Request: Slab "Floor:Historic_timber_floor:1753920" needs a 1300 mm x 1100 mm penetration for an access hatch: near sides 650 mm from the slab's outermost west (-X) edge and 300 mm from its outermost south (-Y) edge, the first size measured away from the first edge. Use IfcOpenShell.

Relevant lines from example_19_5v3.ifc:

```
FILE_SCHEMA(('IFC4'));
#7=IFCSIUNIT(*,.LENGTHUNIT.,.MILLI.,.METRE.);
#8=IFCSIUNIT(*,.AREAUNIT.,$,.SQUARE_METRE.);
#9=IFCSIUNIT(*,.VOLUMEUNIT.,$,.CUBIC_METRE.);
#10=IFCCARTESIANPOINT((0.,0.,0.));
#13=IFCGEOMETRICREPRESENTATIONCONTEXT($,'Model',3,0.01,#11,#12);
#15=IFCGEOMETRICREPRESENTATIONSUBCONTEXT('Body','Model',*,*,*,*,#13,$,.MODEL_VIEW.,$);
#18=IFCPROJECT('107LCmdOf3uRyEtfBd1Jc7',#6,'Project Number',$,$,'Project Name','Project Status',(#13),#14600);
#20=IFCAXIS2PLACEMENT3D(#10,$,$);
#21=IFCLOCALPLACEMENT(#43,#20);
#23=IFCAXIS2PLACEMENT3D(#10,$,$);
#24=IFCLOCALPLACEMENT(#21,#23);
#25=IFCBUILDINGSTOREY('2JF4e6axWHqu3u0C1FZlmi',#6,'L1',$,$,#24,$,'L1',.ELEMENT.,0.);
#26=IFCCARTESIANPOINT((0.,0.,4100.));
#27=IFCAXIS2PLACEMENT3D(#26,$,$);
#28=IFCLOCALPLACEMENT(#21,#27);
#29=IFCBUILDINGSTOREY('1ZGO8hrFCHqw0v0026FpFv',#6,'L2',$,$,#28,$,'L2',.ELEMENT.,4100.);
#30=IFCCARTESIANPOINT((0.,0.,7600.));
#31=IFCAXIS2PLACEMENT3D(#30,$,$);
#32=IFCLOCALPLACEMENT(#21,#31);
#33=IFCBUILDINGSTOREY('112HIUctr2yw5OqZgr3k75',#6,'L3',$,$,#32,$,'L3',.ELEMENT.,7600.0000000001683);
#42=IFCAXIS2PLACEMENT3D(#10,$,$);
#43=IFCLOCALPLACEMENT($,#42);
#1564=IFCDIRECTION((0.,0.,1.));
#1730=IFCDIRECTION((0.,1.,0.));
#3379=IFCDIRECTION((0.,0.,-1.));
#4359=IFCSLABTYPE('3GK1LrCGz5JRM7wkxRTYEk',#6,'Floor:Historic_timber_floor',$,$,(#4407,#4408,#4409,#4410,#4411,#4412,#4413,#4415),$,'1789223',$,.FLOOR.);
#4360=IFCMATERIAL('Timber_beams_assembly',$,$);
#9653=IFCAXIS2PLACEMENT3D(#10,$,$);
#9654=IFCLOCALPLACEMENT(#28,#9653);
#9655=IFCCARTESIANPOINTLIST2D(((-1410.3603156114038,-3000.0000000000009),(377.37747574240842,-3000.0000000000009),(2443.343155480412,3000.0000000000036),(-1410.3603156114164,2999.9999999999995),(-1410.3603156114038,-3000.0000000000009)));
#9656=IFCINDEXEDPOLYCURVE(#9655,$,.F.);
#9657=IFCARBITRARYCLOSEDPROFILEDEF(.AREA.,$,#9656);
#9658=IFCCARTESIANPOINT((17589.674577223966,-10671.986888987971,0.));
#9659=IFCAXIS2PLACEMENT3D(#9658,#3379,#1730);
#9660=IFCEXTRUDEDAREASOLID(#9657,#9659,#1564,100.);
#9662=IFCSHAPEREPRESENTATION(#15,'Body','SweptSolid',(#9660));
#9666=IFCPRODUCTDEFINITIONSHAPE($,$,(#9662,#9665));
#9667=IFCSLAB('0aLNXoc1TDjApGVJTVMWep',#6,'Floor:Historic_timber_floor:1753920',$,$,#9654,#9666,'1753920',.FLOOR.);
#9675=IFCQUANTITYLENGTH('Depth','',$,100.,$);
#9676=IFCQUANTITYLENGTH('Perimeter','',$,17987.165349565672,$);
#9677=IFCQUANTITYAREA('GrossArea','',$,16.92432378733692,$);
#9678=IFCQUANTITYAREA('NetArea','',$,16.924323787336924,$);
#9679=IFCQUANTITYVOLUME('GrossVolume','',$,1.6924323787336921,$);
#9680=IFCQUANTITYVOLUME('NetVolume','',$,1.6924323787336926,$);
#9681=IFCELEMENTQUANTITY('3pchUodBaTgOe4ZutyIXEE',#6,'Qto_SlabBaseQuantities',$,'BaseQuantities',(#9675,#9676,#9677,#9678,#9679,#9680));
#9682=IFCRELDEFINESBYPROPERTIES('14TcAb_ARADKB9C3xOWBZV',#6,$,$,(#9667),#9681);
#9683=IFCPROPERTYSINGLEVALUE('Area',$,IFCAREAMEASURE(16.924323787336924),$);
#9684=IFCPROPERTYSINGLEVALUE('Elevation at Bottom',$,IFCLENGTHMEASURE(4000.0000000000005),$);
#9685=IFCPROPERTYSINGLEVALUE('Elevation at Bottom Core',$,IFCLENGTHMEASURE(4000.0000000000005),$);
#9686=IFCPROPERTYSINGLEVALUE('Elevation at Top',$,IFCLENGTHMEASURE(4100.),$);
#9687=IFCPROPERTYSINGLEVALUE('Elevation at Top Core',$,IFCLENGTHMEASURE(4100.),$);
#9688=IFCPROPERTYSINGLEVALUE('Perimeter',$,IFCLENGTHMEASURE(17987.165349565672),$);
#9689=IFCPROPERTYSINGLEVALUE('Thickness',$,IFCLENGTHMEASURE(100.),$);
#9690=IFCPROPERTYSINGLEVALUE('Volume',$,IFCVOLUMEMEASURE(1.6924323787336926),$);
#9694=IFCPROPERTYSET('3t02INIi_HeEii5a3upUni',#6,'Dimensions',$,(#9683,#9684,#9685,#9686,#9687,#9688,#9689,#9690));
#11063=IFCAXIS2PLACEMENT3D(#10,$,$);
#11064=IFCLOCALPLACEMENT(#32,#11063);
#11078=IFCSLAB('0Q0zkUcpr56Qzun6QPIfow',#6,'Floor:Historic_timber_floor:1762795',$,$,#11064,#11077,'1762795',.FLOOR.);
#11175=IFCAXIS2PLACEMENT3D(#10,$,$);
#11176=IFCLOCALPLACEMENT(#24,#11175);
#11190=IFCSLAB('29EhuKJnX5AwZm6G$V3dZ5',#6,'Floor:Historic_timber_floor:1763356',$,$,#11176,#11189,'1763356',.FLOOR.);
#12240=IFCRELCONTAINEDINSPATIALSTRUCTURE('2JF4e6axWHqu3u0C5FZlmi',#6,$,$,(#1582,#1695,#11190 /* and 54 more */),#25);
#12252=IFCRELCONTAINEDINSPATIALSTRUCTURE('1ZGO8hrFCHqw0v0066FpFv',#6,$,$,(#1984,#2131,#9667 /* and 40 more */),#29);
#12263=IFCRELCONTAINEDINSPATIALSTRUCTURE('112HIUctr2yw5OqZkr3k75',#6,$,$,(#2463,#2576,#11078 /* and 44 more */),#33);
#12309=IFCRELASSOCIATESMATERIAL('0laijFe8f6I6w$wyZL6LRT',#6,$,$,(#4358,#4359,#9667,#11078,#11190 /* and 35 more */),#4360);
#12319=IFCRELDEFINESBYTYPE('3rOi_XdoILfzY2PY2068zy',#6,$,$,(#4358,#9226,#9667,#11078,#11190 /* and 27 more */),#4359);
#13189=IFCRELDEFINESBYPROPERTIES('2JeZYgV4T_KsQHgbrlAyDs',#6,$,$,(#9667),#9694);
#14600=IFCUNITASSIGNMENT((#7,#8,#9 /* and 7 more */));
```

```python
import numpy as np
import ifcopenshell
import ifcopenshell.api.feature
import ifcopenshell.api.geometry
import ifcopenshell.api.pset
import ifcopenshell.api.root
import ifcopenshell.geom
import ifcopenshell.util.element
import ifcopenshell.util.placement
import ifcopenshell.util.representation
import ifcopenshell.util.shape
import ifcopenshell.util.unit

model = ifcopenshell.open("example_19_5v3.ifc")
unit_scale = ifcopenshell.util.unit.calculate_unit_scale(model)
area_scale = ifcopenshell.util.unit.calculate_unit_scale(model, "AREAUNIT")
volume_scale = ifcopenshell.util.unit.calculate_unit_scale(model, "VOLUMEUNIT")
settings = ifcopenshell.geom.settings()


def volume(element):
    """Net volume in cubic metres, openings subtracted."""
    shape = ifcopenshell.geom.create_shape(settings, element)
    return ifcopenshell.util.shape.get_volume(shape.geometry)


slab = model.by_id(9667)
before = volume(slab)

# Extent in the slab's own axes, in metres. The edges named are its -X and -Y sides.
slab_shape = ifcopenshell.geom.create_shape(settings, slab)
vertices = ifcopenshell.util.shape.get_vertices(slab_shape.geometry)
x_min, y_min, bottom = vertices.min(axis=0)
top = vertices[:, 2].max()

opening = ifcopenshell.api.root.create_entity(model, ifc_class="IfcOpeningElement", name="Access hatch opening", predefined_type="OPENING")
context = ifcopenshell.util.representation.get_context(model, "Model", "Body", "MODEL_VIEW")
width, depth = 1.3, 1.1
outline = [(0.0, 0.0), (width, 0.0), (width, depth), (0.0, depth), (0.0, 0.0)]
# Overshoot both faces by 50 mm so the cut is clean.
shape = ifcopenshell.api.geometry.add_slab_representation(
    model, context=context, depth=top - bottom + 0.1, polyline=outline
)
ifcopenshell.api.geometry.assign_representation(model, product=opening, representation=shape)

matrix = ifcopenshell.util.placement.get_local_placement(slab.ObjectPlacement)
matrix[:, 3] = matrix @ np.append(np.array([x_min + 0.65, y_min + 0.3, bottom - 0.05]) / unit_scale, 1.0)
ifcopenshell.api.geometry.edit_object_placement(model, product=opening, matrix=matrix, is_si=False)
ifcopenshell.api.feature.add_feature(model, feature=opening, element=slab)

after = volume(slab)

# Update the slab's stored quantities.
qto = model.by_id(ifcopenshell.util.element.get_pset(slab, "Qto_SlabBaseQuantities", should_inherit=False)["id"])
ifcopenshell.api.pset.edit_qto(model, qto=qto, properties={
    "NetArea": after / (top - bottom) / area_scale,
    "NetVolume": after / volume_scale,
})
pset = model.by_id(ifcopenshell.util.element.get_pset(slab, "Dimensions", should_inherit=False)["id"])
ifcopenshell.api.pset.edit_pset(model, pset=pset, properties={
    "Area": model.create_entity("IfcAreaMeasure", after / (top - bottom) / area_scale),
    "Volume": model.create_entity("IfcVolumeMeasure", after / volume_scale),
})

print(f"slab volume {before:.3f} -> {after:.3f} m3")

model.write("example_19_5v3_v2.ifc")
```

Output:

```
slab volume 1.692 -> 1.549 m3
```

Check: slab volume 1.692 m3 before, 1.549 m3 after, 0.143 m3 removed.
